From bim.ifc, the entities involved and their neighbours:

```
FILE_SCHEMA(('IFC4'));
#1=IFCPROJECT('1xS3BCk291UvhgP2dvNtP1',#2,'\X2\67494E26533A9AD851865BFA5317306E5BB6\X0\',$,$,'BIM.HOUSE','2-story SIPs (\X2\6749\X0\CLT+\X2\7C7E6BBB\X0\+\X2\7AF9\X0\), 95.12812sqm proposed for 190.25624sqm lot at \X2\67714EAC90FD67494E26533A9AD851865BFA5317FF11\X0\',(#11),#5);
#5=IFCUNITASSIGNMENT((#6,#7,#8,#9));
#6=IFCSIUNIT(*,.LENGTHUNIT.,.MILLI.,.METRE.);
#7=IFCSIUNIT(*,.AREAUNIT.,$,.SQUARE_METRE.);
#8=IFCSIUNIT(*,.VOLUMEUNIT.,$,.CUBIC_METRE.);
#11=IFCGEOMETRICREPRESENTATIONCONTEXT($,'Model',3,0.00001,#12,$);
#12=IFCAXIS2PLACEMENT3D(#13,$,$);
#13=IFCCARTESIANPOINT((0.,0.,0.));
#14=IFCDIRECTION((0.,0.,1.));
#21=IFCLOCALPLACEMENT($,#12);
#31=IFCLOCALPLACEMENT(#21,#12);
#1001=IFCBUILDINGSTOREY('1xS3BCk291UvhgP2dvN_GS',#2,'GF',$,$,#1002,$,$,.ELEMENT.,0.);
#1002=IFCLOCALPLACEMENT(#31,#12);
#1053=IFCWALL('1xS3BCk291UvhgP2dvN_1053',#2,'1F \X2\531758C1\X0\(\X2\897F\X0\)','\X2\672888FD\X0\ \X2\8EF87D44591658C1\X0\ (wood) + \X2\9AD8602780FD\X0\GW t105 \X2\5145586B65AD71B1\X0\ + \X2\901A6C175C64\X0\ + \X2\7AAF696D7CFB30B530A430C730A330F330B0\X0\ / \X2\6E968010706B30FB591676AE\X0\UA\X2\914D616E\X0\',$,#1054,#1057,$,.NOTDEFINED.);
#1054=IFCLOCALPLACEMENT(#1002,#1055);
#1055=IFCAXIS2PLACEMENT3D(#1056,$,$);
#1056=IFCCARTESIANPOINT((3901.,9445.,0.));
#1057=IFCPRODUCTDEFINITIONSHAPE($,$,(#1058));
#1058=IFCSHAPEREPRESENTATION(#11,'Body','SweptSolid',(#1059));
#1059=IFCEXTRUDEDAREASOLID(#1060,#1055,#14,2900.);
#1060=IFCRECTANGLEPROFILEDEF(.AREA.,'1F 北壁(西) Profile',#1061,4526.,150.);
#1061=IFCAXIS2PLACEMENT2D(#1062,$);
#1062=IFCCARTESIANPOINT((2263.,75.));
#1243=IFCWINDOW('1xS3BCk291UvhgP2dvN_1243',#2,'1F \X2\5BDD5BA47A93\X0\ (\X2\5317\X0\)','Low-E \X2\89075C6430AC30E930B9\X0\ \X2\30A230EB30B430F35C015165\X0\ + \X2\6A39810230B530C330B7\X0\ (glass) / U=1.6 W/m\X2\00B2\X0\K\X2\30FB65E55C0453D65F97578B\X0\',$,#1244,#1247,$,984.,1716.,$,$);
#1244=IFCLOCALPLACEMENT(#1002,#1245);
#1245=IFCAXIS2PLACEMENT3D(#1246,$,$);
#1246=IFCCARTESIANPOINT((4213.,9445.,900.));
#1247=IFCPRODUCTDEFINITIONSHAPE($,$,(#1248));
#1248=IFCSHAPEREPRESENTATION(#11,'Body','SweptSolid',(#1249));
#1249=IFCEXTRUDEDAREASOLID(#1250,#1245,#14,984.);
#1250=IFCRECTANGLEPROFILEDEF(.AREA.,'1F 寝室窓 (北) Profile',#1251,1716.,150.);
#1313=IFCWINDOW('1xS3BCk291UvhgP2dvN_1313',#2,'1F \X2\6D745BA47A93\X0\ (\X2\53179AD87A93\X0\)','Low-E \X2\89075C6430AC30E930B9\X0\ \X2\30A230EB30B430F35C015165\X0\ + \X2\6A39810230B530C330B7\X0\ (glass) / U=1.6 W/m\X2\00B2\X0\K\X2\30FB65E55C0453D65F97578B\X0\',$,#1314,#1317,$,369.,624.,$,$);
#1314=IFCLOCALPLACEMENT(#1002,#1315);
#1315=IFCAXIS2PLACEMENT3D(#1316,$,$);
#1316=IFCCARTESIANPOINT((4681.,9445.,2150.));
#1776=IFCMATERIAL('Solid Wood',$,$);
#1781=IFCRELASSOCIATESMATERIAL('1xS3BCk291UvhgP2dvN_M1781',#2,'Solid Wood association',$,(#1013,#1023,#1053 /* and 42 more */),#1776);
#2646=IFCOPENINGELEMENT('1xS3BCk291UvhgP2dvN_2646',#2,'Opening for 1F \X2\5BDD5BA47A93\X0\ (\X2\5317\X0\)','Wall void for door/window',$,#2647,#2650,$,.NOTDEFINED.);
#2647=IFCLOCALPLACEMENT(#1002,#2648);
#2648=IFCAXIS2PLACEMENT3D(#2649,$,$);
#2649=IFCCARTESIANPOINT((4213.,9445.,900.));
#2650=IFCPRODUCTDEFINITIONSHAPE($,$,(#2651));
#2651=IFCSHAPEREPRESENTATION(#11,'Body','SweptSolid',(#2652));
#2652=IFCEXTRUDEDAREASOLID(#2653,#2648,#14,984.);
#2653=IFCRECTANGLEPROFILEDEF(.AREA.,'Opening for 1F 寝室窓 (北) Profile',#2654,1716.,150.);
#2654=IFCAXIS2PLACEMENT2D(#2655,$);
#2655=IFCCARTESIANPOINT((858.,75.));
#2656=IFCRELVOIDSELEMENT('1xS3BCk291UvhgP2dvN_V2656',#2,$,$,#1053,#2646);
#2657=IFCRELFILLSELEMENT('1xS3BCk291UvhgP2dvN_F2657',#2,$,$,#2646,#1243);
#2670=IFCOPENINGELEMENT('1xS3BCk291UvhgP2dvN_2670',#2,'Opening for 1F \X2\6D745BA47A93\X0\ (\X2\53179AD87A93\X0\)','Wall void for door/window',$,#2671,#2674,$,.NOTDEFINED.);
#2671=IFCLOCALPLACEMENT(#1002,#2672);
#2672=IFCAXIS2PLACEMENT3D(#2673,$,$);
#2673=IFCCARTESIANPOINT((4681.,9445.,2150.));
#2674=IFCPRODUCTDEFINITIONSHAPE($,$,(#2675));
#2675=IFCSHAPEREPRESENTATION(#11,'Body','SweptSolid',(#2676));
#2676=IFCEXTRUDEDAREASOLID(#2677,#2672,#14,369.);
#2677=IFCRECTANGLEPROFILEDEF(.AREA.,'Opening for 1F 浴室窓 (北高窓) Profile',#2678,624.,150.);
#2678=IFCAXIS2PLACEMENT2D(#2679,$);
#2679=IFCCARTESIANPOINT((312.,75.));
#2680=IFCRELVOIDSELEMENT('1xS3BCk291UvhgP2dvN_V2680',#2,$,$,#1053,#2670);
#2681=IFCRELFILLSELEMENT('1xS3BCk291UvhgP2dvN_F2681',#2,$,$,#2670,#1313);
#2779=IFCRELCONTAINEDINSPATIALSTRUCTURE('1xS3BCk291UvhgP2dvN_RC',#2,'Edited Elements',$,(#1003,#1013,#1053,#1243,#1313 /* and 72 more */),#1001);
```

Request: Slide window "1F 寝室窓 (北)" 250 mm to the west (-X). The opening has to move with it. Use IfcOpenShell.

```python
import ifcopenshell
import ifcopenshell.api.geometry
import ifcopenshell.util.placement
import ifcopenshell.util.unit

model = ifcopenshell.open("bim.ifc")
unit_scale = ifcopenshell.util.unit.calculate_unit_scale(model)

window = model.by_id(1243)
opening = window.FillsVoids[0].RelatingOpeningElement
wall = opening.VoidsElements[0].RelatingBuildingElement

wall_matrix = ifcopenshell.util.placement.get_local_placement(wall.ObjectPlacement)
shift = wall_matrix[:3, 0] * -0.25 / unit_scale
before = ifcopenshell.util.placement.get_local_placement(window.ObjectPlacement)[:3, 3].copy()

# The window is not placed relative to its opening, so move both.
for product in (opening, window):
    matrix = ifcopenshell.util.placement.get_local_placement(product.ObjectPlacement)
    matrix[:3, 3] += shift
    ifcopenshell.api.geometry.edit_object_placement(model, product=product, matrix=matrix, is_si=False)

after = ifcopenshell.util.placement.get_local_placement(window.ObjectPlacement)[:3, 3]
print("window moved by", (after - before).round(3) + 0.0)

model.write("bim_updated.ifc")
```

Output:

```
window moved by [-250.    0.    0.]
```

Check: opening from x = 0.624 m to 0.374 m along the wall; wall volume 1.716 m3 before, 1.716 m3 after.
